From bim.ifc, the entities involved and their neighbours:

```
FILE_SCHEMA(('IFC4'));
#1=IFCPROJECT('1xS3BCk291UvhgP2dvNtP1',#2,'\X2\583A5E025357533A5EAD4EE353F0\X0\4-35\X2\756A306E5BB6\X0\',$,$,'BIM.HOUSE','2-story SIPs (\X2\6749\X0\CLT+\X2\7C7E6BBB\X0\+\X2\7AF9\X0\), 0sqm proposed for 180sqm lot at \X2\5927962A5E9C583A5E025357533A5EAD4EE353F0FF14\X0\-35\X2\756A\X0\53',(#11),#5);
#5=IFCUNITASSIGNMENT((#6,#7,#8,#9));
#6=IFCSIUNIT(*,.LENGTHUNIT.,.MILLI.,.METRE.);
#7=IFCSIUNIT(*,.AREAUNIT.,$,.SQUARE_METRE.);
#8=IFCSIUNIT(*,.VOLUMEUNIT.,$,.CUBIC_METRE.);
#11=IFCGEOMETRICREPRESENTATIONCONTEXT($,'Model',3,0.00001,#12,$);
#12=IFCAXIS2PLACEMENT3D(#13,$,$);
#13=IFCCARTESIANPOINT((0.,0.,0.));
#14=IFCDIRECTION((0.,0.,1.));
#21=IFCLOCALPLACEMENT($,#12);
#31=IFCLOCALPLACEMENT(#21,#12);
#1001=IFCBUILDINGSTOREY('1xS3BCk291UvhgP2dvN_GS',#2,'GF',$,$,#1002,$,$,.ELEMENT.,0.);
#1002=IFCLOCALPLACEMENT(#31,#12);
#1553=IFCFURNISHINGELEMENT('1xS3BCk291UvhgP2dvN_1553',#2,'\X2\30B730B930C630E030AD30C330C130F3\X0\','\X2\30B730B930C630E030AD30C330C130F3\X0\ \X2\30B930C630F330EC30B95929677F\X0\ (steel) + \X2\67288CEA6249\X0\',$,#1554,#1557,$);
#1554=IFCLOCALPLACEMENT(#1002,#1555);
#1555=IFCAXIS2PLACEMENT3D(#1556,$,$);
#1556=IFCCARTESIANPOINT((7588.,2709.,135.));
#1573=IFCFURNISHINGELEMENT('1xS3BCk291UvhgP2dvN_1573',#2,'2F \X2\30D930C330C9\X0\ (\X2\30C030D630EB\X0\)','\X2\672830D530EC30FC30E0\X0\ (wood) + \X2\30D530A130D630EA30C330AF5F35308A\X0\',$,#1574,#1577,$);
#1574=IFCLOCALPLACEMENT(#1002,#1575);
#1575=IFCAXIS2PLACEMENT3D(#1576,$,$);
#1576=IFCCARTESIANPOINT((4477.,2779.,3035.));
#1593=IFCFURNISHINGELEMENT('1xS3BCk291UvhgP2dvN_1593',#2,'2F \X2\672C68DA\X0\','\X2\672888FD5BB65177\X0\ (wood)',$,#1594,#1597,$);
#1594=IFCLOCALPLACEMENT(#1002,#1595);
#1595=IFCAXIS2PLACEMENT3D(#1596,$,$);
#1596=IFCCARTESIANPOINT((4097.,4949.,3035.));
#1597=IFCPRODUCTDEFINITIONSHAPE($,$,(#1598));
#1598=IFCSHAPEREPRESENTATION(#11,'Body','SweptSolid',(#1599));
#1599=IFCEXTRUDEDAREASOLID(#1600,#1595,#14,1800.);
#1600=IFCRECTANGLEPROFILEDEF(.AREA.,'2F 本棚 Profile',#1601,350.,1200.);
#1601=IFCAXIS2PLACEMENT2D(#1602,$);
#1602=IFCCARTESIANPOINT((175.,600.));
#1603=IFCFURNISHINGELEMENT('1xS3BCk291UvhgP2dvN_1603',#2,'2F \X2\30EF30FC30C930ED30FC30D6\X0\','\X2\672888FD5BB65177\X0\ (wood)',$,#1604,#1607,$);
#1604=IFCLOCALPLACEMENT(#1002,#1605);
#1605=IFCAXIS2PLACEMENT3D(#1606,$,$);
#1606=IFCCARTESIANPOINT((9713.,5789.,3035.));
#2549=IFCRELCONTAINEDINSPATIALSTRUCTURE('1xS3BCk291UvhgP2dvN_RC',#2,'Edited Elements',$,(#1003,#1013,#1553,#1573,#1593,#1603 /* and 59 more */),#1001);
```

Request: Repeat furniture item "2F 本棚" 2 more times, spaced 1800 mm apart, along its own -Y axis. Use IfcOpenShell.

```python
import ifcopenshell
import ifcopenshell.api.geometry
import ifcopenshell.api.root
import ifcopenshell.util.element
import ifcopenshell.util.placement

model = ifcopenshell.open("bim.ifc")


def reuse_history(source, copy):
    """copy_class also copies each property set's owner history, people and application; keep the originals."""
    for rel in copy.IsDefinedBy:
        if rel.is_a("IfcRelDefinesByProperties") and (history := rel.RelatingPropertyDefinition.OwnerHistory):
            rel.RelatingPropertyDefinition.OwnerHistory = source.OwnerHistory
            ifcopenshell.util.element.remove_deep2(model, history)


source = model.by_id(1593)
base = ifcopenshell.util.placement.get_local_placement(source.ObjectPlacement)
step = -base[:3, 1] * 1800.0

for i in range(1, 3):
    copy = ifcopenshell.api.root.copy_class(model, product=source)
    copy.Representation = ifcopenshell.util.element.copy_deep(
        model, source.Representation, exclude=["IfcGeometricRepresentationContext", "IfcRepresentationMap"]
    )
    reuse_history(source, copy)
    matrix = base.copy()
    matrix[:3, 3] += i * step
    print("added at", matrix[:3, 3].round(3) + 0.0)
    ifcopenshell.api.geometry.edit_object_placement(model, product=copy, matrix=matrix, is_si=False)

model.write("bim_edited.ifc")
```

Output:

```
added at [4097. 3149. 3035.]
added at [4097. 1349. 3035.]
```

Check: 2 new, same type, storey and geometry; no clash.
